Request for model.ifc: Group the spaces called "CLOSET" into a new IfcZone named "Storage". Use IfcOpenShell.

First a look at what the model holds.

```python
import ifcopenshell

model = ifcopenshell.open("model.ifc")
print(model.schema)
seen = {}
for space in model.by_type("IfcSpace"):
    seen[space.LongName] = seen.get(space.LongName, 0) + 1
for name, count in sorted(seen.items(), key=str):
    print(count, "x", name)
print("zones:", [z.Name for z in model.by_type("IfcZone")][:20])
```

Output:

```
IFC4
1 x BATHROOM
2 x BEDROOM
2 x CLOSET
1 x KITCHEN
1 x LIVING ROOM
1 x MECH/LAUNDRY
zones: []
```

```python
import ifcopenshell
import ifcopenshell.api.group
import ifcopenshell.api.root

model = ifcopenshell.open("model.ifc")

names = {"CLOSET"}
spaces = [s for s in model.by_type("IfcSpace") if s.LongName in names]

zone = ifcopenshell.api.root.create_entity(model, ifc_class="IfcZone", name="Storage")
ifcopenshell.api.group.assign_group(model, products=spaces, group=zone)
print(len(spaces), "spaces in", zone.Name)

model.write("model_updated.ifc")
```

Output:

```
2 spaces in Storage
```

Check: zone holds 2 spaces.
